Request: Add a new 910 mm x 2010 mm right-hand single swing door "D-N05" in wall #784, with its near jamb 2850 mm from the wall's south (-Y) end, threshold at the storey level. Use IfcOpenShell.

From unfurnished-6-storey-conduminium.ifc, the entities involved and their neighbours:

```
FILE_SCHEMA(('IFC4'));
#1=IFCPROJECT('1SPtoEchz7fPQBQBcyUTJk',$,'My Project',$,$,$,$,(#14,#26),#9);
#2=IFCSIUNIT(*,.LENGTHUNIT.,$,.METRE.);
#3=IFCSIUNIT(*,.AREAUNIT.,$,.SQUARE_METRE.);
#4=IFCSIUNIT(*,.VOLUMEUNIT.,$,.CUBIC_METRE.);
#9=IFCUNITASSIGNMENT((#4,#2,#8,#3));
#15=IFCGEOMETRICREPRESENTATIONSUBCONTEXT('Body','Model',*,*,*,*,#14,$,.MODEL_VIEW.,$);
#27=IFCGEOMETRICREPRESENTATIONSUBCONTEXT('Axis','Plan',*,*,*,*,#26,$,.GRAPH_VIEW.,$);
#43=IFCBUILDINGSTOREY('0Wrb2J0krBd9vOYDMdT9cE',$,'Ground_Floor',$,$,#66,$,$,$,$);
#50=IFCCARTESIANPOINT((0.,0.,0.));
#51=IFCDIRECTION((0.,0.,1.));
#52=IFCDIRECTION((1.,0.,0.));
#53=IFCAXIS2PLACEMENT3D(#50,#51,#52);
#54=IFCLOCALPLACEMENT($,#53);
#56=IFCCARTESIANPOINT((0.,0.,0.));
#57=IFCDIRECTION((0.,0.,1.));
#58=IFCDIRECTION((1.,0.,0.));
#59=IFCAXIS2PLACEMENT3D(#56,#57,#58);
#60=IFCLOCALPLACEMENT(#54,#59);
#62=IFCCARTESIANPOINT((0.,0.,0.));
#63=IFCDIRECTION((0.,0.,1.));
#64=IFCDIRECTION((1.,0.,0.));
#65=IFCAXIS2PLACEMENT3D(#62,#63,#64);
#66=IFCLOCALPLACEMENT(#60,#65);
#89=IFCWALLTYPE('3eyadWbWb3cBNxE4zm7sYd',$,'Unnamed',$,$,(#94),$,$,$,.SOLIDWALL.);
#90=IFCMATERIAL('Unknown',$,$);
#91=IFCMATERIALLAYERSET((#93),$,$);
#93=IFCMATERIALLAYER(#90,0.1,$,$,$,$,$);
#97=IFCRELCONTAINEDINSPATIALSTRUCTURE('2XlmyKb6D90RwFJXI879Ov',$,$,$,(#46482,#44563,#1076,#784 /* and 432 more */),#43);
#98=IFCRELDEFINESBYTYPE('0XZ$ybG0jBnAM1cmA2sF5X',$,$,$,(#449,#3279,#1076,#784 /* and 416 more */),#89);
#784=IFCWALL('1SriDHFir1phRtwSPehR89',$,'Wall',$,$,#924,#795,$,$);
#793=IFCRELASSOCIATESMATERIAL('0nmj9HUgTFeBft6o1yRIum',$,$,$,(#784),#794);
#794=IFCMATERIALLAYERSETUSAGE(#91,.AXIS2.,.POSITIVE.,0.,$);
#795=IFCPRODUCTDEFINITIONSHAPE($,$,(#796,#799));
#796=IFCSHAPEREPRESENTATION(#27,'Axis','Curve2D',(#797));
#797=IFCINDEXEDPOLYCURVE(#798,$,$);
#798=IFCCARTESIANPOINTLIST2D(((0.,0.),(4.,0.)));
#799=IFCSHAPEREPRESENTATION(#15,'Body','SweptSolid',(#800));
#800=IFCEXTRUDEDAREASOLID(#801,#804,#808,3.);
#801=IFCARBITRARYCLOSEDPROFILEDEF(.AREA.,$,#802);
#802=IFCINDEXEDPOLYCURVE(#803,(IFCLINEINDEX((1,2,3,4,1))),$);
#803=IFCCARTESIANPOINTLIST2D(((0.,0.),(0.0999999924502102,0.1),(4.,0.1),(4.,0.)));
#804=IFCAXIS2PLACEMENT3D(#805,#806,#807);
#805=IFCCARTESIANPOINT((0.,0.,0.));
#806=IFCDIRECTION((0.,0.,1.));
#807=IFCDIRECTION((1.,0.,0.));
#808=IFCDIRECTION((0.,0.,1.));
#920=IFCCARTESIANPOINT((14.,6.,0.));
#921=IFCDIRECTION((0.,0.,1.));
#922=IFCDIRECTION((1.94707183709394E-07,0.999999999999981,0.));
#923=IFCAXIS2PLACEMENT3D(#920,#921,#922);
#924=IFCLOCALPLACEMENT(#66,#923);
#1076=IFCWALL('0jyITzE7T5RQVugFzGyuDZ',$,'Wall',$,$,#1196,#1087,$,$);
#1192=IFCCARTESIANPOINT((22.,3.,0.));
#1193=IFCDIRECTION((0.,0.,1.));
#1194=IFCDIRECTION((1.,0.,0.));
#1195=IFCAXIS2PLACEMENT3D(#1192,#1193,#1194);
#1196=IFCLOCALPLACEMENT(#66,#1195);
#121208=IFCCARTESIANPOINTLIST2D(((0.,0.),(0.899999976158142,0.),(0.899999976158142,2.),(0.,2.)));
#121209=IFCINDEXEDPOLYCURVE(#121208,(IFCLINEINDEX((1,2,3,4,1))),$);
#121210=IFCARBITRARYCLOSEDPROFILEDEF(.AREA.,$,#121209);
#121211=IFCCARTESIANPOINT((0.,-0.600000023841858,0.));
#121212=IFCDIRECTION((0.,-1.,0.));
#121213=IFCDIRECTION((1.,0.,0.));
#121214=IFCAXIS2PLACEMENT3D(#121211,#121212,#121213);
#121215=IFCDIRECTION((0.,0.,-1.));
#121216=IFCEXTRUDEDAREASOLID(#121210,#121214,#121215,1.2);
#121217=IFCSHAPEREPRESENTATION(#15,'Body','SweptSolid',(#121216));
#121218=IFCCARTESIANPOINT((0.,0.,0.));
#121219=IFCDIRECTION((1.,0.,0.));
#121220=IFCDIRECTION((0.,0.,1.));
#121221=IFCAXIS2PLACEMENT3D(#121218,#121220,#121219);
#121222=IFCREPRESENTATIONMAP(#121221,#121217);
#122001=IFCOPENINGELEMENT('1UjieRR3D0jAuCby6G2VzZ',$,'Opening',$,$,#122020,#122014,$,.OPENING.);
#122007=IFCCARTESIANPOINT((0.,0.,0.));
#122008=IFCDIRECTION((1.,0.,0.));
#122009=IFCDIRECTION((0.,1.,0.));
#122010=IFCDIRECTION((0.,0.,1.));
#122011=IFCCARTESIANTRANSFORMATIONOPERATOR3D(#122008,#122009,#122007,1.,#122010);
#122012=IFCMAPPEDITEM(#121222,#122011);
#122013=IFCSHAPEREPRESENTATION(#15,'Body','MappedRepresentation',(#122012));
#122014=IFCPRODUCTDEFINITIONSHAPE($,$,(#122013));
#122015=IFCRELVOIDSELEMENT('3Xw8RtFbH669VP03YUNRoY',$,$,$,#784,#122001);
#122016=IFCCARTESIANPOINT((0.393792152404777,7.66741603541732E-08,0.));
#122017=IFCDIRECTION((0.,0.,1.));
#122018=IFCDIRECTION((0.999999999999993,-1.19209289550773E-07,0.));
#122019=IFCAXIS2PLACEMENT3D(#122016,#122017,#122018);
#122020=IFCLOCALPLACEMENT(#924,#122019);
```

```python
import numpy as np
import ifcopenshell
import ifcopenshell.api.feature
import ifcopenshell.api.geometry
import ifcopenshell.api.root
import ifcopenshell.api.spatial
import ifcopenshell.geom
import ifcopenshell.util.element
import ifcopenshell.util.placement
import ifcopenshell.util.representation
import ifcopenshell.util.shape
import ifcopenshell.util.unit

model = ifcopenshell.open("unfurnished-6-storey-conduminium.ifc")
unit_scale = ifcopenshell.util.unit.calculate_unit_scale(model)
settings = ifcopenshell.geom.settings()


def volume(element):
    """Net volume in cubic metres, openings subtracted."""
    shape = ifcopenshell.geom.create_shape(settings, element)
    return ifcopenshell.util.shape.get_volume(shape.geometry)


wall = model.by_guid("1SriDHFir1phRtwSPehR89")
storey = ifcopenshell.util.element.get_container(wall, ifc_class="IfcBuildingStorey")
context = ifcopenshell.util.representation.get_context(model, "Model", "Body", "MODEL_VIEW")
before = volume(wall)

width, height, from_end, sill = 0.91, 2.01, 2.85, 0.0  # metres

# The wall runs along its own X axis, and the end named is its -X end.
wall_shape = ifcopenshell.geom.create_shape(settings, wall)
x, y, z = ifcopenshell.util.shape.get_vertices(wall_shape.geometry).T
start = x.min() + from_end
face, thickness = float(y.min()), float(y.max() - y.min())
wall_matrix = ifcopenshell.util.placement.get_local_placement(wall.ObjectPlacement)
level = ifcopenshell.util.placement.get_local_placement(storey.ObjectPlacement)[2, 3]


def in_wall(x, y):
    """Placement at x, y metres in the wall's axes, at sill height."""
    matrix = wall_matrix.copy()
    matrix[:, 3] = wall_matrix @ np.array([x / unit_scale, y / unit_scale, 0.0, 1.0])
    matrix[2, 3] = level + sill / unit_scale
    return matrix


# Opening: a box that overshoots both wall faces by 50 mm.
opening = ifcopenshell.api.root.create_entity(model, ifc_class="IfcOpeningElement", predefined_type="OPENING")
box = ifcopenshell.api.geometry.add_wall_representation(
    model, context=context, length=width, height=height, thickness=thickness + 0.1
)
ifcopenshell.api.geometry.assign_representation(model, product=opening, representation=box)
ifcopenshell.api.geometry.edit_object_placement(model, product=opening, matrix=in_wall(start, face - 0.05), is_si=False)
ifcopenshell.api.feature.add_feature(model, feature=opening, element=wall)

door = ifcopenshell.api.root.create_entity(model, ifc_class="IfcDoor", name="D-N05", predefined_type="DOOR")
door.OverallWidth, door.OverallHeight = width / unit_scale, height / unit_scale
door.OperationType = "SINGLE_SWING_RIGHT"
body = ifcopenshell.api.geometry.add_door_representation(
    model,
    context=context,
    overall_width=door.OverallWidth,
    overall_height=door.OverallHeight,
    operation_type="SINGLE_SWING_RIGHT",
    lining_properties={"LiningDepth": thickness / unit_scale, "ThresholdDepth": thickness / unit_scale},
)
ifcopenshell.api.geometry.assign_representation(model, product=door, representation=body)
ifcopenshell.api.spatial.assign_container(model, products=[door], relating_structure=storey)
ifcopenshell.api.feature.add_filling(model, opening=opening, element=door)

# The lining spans the wall, so the door starts at the wall face.
ifcopenshell.api.geometry.edit_object_placement(model, product=door, matrix=in_wall(start, face), is_si=False)

after = volume(wall)

print(f"wall volume {before:.3f} -> {after:.3f} m3")

model.write("unfurnished-6-storey-conduminium_rev.ifc")
```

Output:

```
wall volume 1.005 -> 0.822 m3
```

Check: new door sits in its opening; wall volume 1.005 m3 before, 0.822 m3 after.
